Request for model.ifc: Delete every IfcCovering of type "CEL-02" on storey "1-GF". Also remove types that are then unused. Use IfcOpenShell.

First a look at what the model holds.

```python
import ifcopenshell
import ifcopenshell.util.element

model = ifcopenshell.open("model.ifc")
print(model.schema)
storey = next(s for s in model.by_type("IfcBuildingStorey") if s.Name == "1-GF")
coverings = [e for e in ifcopenshell.util.element.get_decomposition(storey) if e.is_a("IfcCovering")]
seen = {}
for e in coverings:
    element_type = ifcopenshell.util.element.get_type(e)
    name = element_type.Name if element_type not in (None, e) else None
    seen[name] = seen.get(name, 0) + 1
for name, count in sorted(seen.items(), key=str):
    print(count, "x", name)
```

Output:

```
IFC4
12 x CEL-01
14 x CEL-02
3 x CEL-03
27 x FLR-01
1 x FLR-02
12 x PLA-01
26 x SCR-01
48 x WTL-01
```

```python
import ifcopenshell
import ifcopenshell.api.root
import ifcopenshell.util.element

model = ifcopenshell.open("model.ifc")

storey = next(s for s in model.by_type("IfcBuildingStorey") if s.Name == "1-GF")
coverings = [e for e in ifcopenshell.util.element.get_decomposition(storey) if e.is_a("IfcCovering")]
targets = [e for e in coverings if (t := ifcopenshell.util.element.get_type(e)) not in (None, e) and t.Name == "CEL-02"]
types = {ifcopenshell.util.element.get_type(e) for e in targets} - {None, *targets}

for e in targets:
    ifcopenshell.api.root.remove_product(model, product=e)
print(len(targets), "removed")

unused = [t for t in types if not ifcopenshell.util.element.get_types(t)]
for t in unused:
    ifcopenshell.api.root.remove_product(model, product=t)
print(len(unused), "unused types removed")

model.write("model-out.ifc")
```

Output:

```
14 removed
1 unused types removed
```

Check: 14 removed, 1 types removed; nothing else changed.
